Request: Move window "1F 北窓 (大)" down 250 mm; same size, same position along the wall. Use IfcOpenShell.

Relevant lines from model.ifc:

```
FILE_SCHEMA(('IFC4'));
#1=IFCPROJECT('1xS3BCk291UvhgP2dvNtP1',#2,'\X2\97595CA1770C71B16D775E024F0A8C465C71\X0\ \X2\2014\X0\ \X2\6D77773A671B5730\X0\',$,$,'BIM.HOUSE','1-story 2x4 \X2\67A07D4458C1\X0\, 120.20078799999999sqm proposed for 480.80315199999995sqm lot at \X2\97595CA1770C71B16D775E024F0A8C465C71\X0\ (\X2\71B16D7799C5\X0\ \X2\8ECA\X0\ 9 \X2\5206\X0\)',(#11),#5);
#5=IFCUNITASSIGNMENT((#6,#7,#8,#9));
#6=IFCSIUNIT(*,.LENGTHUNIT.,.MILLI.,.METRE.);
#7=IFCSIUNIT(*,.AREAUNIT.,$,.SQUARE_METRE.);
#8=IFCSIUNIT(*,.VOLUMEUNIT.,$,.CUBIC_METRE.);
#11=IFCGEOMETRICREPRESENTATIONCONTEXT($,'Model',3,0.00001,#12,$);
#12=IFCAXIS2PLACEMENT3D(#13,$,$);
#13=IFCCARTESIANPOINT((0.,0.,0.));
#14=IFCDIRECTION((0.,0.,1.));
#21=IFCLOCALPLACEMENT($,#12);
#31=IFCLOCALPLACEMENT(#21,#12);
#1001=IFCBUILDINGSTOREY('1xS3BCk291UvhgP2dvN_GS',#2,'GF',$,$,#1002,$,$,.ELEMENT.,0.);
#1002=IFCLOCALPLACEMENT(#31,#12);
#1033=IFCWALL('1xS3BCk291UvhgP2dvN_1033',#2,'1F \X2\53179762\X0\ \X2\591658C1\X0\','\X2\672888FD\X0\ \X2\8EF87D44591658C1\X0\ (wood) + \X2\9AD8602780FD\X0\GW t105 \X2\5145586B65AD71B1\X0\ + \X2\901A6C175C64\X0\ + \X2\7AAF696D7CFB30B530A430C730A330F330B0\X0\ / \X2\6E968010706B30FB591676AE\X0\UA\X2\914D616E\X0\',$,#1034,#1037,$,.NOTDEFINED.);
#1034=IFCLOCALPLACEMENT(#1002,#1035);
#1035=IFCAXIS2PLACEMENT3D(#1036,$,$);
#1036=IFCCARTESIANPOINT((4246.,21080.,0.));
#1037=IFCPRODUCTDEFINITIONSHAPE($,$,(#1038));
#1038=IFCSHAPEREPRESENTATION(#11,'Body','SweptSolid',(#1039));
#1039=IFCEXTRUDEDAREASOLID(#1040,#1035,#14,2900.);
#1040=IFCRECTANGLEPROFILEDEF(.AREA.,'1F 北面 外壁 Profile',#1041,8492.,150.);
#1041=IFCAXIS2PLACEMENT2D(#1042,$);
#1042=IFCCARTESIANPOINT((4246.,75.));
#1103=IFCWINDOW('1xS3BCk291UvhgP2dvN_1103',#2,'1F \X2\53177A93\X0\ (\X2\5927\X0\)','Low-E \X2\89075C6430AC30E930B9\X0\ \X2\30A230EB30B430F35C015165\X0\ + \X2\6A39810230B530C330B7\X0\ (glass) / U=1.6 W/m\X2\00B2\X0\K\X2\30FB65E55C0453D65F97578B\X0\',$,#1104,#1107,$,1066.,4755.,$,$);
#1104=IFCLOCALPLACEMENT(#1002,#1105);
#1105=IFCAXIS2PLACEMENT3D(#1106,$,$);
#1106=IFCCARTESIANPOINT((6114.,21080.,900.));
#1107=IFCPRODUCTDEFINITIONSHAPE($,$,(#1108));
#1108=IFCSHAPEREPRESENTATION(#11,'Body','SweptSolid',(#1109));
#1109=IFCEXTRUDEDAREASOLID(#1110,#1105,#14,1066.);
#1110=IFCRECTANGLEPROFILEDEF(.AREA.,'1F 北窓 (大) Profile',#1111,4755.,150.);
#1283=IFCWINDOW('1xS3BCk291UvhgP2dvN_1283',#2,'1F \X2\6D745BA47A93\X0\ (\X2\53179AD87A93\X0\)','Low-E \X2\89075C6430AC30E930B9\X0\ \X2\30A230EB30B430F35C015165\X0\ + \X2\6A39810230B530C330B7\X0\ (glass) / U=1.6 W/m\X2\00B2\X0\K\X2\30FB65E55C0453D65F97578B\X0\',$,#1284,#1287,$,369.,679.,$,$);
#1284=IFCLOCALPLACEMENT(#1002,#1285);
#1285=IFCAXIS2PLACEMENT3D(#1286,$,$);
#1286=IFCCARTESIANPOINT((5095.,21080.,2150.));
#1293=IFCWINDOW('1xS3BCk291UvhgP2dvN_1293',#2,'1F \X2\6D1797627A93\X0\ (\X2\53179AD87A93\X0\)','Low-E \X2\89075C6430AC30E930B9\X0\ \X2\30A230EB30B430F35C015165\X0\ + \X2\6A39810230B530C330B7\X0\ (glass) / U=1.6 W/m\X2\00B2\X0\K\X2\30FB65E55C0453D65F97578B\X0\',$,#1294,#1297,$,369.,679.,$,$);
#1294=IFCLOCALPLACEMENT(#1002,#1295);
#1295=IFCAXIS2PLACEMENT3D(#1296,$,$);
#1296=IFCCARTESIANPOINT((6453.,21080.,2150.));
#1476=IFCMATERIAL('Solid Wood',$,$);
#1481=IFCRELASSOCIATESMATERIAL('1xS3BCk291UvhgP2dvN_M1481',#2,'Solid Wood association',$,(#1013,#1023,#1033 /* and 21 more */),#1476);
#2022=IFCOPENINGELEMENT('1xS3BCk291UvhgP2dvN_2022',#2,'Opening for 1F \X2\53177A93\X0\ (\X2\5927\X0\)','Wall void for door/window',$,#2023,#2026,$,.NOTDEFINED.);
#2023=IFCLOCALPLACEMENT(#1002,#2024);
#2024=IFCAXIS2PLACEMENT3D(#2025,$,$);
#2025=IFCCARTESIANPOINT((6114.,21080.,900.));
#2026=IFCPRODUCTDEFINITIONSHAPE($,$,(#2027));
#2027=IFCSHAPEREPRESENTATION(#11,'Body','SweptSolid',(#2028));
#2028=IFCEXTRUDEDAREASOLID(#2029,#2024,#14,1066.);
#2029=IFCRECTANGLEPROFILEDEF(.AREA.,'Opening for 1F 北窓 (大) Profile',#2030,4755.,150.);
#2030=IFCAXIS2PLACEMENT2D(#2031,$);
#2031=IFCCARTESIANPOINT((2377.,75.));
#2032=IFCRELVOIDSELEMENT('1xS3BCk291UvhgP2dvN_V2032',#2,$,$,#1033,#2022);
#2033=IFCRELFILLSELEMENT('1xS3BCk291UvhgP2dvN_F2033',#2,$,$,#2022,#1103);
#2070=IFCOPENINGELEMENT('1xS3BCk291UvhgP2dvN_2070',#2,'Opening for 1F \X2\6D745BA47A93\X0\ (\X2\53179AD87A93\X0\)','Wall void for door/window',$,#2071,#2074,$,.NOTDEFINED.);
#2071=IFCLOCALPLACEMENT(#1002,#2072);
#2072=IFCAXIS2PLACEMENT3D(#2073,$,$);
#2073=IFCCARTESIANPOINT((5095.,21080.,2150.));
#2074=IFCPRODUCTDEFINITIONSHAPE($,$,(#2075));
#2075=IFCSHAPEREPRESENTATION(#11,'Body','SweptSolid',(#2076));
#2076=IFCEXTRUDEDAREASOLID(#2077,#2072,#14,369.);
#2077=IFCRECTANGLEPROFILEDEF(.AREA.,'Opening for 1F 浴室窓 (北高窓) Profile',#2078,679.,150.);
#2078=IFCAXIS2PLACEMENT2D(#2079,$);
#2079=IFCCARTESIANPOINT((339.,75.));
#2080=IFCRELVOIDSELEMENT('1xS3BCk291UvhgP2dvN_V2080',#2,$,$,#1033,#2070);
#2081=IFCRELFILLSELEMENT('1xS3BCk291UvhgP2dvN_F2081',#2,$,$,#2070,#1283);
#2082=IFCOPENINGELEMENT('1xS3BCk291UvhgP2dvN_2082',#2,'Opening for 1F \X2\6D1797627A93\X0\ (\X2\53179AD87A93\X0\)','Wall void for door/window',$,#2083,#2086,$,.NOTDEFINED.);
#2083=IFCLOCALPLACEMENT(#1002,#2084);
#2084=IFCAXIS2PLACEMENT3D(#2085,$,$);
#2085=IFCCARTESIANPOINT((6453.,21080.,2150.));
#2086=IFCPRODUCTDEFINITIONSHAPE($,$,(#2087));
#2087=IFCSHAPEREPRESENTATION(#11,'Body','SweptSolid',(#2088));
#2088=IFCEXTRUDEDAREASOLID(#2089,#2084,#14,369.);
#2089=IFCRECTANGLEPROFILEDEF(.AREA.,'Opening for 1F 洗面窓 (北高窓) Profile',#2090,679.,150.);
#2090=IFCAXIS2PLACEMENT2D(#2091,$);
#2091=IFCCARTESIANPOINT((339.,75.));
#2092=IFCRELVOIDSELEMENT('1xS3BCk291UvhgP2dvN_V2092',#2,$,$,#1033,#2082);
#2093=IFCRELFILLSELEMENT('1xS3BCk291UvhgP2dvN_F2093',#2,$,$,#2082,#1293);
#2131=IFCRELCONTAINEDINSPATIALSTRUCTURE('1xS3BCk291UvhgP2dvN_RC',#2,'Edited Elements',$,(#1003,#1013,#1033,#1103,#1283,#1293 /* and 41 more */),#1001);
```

```python
import numpy as np
import ifcopenshell
import ifcopenshell.api.geometry
import ifcopenshell.util.placement
import ifcopenshell.util.unit

model = ifcopenshell.open("model.ifc")
unit_scale = ifcopenshell.util.unit.calculate_unit_scale(model)

window = model.by_guid("1xS3BCk291UvhgP2dvN_1103")
opening = window.FillsVoids[0].RelatingOpeningElement
dz = -0.25 / unit_scale

shift = np.array([0.0, 0.0, dz])
# The window is not placed relative to its opening, so move both.
for product in (opening, window):
    matrix = ifcopenshell.util.placement.get_local_placement(product.ObjectPlacement)
    matrix[:3, 3] += shift
    ifcopenshell.api.geometry.edit_object_placement(model, product=product, matrix=matrix, is_si=False)

print(f"moved by {dz * unit_scale:+.3f} m")

model.write("model-out.ifc")
```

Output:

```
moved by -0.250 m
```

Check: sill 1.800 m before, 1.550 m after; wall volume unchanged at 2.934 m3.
